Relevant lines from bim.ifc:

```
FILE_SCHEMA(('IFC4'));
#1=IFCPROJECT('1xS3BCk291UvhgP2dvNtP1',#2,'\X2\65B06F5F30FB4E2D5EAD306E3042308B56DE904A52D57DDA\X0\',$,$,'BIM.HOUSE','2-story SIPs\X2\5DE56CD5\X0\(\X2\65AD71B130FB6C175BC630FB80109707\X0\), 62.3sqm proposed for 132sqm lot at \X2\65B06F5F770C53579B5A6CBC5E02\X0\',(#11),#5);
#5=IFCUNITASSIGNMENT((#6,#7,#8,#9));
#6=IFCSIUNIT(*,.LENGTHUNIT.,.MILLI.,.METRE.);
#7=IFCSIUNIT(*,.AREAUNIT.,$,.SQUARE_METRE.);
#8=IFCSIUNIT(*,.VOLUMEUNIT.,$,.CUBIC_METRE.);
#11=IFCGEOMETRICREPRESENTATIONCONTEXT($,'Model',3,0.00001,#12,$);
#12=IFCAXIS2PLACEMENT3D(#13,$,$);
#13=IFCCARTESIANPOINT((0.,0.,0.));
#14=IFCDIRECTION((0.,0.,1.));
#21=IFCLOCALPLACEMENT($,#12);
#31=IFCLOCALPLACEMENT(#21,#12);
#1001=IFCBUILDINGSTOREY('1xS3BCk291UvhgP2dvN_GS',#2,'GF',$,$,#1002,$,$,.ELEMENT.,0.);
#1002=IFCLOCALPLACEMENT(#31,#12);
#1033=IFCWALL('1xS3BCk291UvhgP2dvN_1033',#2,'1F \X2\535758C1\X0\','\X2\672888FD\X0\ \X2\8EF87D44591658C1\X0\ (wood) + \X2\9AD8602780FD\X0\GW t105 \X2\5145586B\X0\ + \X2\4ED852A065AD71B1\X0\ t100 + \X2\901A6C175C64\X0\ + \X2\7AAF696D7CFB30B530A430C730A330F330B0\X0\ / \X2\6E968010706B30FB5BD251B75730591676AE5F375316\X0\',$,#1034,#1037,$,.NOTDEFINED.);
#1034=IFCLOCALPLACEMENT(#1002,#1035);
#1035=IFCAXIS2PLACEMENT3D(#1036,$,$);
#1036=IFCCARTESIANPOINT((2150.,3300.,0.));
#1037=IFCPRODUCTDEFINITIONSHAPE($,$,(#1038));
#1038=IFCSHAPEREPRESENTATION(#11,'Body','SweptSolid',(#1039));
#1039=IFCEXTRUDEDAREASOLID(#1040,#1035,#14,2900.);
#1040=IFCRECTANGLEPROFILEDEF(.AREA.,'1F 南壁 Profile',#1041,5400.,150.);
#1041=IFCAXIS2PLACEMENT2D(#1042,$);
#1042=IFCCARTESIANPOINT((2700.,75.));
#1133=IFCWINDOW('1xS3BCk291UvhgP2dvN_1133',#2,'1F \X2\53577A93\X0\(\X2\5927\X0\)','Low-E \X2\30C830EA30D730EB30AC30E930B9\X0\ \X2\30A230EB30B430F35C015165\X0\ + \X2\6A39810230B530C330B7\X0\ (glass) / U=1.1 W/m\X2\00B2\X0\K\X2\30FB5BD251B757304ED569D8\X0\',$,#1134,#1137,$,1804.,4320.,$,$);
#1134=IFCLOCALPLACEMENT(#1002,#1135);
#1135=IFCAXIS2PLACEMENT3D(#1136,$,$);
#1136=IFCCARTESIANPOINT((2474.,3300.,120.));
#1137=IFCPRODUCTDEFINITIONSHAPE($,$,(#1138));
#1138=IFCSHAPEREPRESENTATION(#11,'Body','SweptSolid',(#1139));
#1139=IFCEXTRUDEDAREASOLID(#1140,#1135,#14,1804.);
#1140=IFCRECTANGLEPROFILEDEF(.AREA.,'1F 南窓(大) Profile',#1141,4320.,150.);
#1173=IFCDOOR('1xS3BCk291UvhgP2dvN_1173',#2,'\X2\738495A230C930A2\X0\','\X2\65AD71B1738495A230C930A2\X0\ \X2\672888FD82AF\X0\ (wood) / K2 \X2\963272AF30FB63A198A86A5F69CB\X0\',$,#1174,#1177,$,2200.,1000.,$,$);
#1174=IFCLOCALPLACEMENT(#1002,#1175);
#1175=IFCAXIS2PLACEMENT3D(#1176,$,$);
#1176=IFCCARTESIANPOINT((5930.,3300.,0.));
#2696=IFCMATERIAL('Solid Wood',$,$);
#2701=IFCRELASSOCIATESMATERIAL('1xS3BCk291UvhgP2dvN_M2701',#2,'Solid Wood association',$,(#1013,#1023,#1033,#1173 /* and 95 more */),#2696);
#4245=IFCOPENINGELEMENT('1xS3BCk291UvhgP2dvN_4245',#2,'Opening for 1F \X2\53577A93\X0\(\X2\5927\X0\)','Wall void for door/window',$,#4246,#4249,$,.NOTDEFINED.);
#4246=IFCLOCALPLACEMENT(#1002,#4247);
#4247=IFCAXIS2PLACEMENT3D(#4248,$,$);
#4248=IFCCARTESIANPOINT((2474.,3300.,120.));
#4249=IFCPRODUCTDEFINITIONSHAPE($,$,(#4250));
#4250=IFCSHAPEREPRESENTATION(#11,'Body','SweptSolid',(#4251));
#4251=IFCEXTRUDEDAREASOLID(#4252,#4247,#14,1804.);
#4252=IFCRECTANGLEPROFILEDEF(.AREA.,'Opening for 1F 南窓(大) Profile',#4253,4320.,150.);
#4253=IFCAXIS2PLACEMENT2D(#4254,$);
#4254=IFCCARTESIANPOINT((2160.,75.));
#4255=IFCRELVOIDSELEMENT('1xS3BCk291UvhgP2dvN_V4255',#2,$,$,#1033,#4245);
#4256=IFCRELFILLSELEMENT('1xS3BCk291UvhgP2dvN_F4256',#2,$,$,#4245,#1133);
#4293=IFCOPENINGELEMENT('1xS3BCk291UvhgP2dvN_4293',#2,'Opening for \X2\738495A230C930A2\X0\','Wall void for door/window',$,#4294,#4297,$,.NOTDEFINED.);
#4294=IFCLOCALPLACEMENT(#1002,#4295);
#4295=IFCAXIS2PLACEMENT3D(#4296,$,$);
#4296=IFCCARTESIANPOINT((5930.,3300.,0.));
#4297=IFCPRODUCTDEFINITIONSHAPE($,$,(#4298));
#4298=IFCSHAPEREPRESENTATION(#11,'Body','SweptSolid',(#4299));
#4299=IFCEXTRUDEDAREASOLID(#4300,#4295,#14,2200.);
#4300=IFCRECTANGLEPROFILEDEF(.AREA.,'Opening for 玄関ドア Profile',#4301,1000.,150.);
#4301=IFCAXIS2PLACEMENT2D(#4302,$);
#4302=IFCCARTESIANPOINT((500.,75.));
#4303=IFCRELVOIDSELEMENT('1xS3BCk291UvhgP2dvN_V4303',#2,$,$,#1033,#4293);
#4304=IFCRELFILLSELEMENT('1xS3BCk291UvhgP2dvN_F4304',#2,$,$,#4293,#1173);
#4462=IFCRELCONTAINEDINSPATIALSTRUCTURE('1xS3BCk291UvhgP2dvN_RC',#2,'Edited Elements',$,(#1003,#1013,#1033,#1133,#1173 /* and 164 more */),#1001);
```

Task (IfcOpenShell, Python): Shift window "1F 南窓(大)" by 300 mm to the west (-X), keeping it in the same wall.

```python
import ifcopenshell
import ifcopenshell.api.geometry
import ifcopenshell.util.placement
import ifcopenshell.util.unit

model = ifcopenshell.open("bim.ifc")
unit_scale = ifcopenshell.util.unit.calculate_unit_scale(model)

window = model.by_id(1133)
opening = window.FillsVoids[0].RelatingOpeningElement
wall = opening.VoidsElements[0].RelatingBuildingElement

wall_matrix = ifcopenshell.util.placement.get_local_placement(wall.ObjectPlacement)
shift = wall_matrix[:3, 0] * -0.3 / unit_scale
before = ifcopenshell.util.placement.get_local_placement(window.ObjectPlacement)[:3, 3].copy()

# The window is not placed relative to its opening, so move both.
for product in (opening, window):
    matrix = ifcopenshell.util.placement.get_local_placement(product.ObjectPlacement)
    matrix[:3, 3] += shift
    ifcopenshell.api.geometry.edit_object_placement(model, product=product, matrix=matrix, is_si=False)

after = ifcopenshell.util.placement.get_local_placement(window.ObjectPlacement)[:3, 3]
print("window moved by", (after - before).round(3) + 0.0)

model.write("bim_rev.ifc")
```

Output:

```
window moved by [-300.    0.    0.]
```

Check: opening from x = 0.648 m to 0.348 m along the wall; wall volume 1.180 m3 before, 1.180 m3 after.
